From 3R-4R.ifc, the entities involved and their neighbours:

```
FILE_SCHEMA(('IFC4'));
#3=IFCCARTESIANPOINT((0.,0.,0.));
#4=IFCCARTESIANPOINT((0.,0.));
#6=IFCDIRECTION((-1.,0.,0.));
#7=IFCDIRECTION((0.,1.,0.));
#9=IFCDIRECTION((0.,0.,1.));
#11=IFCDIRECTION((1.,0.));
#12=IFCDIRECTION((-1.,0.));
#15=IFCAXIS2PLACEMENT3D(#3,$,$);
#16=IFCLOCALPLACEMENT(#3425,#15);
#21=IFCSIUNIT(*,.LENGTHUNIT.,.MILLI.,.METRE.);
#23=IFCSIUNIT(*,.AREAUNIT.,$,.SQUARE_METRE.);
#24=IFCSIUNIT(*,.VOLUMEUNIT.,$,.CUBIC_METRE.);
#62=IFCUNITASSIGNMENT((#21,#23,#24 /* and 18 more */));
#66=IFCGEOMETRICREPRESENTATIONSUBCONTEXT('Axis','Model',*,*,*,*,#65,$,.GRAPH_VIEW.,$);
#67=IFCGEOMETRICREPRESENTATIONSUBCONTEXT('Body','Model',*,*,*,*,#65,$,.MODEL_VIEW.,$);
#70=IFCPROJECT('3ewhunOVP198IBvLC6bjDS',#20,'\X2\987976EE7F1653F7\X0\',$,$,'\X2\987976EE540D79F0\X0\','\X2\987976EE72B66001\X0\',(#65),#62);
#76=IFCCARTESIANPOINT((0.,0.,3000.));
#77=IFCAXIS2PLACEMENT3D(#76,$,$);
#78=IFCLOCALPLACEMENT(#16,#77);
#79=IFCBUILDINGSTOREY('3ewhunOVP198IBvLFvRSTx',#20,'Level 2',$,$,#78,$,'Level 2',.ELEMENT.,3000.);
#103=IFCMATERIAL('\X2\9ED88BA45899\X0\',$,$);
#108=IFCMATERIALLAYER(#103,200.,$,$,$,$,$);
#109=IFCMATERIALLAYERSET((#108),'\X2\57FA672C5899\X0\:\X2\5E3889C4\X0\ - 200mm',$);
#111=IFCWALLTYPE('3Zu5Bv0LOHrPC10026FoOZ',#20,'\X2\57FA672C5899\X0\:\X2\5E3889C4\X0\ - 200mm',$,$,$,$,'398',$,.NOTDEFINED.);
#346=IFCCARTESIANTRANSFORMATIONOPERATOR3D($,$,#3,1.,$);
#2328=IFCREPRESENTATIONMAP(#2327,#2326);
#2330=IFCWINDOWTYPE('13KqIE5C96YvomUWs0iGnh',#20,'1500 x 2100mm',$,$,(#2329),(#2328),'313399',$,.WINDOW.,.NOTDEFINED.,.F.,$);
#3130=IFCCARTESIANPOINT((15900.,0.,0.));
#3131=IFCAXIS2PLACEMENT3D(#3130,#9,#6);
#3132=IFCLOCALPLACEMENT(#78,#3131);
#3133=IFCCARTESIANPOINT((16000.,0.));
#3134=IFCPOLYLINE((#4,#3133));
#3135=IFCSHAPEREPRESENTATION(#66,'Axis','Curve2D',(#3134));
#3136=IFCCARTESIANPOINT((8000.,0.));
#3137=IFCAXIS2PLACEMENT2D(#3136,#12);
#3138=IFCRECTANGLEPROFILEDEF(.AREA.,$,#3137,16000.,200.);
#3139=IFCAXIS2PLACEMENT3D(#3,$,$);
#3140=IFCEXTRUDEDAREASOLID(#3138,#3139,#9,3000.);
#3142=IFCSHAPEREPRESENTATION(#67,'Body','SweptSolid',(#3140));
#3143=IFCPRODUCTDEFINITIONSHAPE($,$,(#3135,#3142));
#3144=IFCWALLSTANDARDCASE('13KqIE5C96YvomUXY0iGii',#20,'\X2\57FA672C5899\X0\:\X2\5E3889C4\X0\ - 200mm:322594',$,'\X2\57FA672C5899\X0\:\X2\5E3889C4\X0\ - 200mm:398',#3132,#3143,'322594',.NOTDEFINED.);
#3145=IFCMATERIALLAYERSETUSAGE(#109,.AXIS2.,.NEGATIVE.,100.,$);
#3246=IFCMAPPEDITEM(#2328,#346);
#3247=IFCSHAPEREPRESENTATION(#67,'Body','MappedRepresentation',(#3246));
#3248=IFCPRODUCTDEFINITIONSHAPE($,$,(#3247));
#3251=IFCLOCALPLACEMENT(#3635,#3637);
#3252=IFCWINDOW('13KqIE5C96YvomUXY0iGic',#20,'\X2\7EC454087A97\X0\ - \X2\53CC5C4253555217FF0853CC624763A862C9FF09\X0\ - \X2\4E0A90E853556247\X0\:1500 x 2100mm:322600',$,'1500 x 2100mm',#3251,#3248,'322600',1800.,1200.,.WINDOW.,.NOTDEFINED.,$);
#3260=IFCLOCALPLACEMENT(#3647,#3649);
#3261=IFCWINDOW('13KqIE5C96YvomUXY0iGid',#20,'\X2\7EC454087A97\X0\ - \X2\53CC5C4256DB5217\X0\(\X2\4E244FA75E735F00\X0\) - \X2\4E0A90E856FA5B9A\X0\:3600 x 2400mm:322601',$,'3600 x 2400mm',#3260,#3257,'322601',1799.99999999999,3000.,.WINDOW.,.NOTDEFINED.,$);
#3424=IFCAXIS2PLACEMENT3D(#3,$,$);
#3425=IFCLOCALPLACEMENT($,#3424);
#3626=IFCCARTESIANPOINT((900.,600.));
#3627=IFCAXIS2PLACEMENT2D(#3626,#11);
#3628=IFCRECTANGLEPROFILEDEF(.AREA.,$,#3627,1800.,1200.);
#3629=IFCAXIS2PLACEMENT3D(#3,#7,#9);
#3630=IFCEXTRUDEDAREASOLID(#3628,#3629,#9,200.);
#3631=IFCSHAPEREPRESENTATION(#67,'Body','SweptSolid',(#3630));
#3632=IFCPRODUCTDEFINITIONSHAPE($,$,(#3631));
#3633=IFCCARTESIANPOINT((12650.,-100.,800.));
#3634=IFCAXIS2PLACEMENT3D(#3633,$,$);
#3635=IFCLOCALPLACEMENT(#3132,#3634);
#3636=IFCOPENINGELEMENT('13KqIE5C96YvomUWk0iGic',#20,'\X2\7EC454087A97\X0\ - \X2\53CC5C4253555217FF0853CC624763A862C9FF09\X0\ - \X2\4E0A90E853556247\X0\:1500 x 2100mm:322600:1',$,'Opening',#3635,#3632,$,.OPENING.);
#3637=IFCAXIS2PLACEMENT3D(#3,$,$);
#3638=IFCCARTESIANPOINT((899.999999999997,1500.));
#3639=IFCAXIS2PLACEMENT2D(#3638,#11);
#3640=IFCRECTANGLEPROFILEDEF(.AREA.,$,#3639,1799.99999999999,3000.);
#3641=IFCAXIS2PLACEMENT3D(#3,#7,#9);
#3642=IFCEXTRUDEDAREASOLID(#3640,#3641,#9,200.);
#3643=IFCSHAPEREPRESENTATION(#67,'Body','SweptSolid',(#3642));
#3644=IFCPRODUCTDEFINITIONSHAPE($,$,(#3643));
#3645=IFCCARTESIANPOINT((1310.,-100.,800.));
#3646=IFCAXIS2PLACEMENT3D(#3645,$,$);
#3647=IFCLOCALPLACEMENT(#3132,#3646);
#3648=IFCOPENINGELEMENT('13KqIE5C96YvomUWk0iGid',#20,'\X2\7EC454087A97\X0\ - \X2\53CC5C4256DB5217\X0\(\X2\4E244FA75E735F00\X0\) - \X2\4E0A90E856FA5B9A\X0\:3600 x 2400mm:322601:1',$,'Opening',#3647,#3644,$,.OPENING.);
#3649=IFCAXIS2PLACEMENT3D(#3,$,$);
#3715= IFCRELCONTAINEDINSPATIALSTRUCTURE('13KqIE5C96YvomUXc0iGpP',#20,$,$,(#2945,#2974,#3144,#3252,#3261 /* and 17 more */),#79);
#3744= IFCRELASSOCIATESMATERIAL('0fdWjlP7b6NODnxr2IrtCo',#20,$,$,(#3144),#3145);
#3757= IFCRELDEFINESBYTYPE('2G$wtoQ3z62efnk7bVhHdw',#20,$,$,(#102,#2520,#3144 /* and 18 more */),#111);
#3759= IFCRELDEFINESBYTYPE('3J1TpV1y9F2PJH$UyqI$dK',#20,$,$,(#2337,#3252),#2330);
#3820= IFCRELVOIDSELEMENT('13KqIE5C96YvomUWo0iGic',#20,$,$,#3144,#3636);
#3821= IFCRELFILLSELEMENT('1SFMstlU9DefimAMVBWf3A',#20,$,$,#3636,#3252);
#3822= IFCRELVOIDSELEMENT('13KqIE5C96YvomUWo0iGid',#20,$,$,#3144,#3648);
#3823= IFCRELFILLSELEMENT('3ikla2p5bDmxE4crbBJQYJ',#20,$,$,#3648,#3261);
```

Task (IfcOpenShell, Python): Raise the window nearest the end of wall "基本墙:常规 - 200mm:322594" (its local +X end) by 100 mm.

```python
import numpy as np
import ifcopenshell
import ifcopenshell.api.geometry
import ifcopenshell.util.placement
import ifcopenshell.util.unit

model = ifcopenshell.open("3R-4R.ifc")
unit_scale = ifcopenshell.util.unit.calculate_unit_scale(model)

window = model.by_id(3252)
opening = window.FillsVoids[0].RelatingOpeningElement
dz = 100.0

shift = np.array([0.0, 0.0, dz])
# The window is placed relative to its opening, so it follows when the opening moves.
matrix = ifcopenshell.util.placement.get_local_placement(opening.ObjectPlacement)
matrix[:3, 3] += shift
ifcopenshell.api.geometry.edit_object_placement(
    model, product=opening, matrix=matrix, is_si=False, should_transform_children=True
)

print(f"moved by {dz * unit_scale:+.3f} m")

model.write("3R-4R_v2.ifc")
```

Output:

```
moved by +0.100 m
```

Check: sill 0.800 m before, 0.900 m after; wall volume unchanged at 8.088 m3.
